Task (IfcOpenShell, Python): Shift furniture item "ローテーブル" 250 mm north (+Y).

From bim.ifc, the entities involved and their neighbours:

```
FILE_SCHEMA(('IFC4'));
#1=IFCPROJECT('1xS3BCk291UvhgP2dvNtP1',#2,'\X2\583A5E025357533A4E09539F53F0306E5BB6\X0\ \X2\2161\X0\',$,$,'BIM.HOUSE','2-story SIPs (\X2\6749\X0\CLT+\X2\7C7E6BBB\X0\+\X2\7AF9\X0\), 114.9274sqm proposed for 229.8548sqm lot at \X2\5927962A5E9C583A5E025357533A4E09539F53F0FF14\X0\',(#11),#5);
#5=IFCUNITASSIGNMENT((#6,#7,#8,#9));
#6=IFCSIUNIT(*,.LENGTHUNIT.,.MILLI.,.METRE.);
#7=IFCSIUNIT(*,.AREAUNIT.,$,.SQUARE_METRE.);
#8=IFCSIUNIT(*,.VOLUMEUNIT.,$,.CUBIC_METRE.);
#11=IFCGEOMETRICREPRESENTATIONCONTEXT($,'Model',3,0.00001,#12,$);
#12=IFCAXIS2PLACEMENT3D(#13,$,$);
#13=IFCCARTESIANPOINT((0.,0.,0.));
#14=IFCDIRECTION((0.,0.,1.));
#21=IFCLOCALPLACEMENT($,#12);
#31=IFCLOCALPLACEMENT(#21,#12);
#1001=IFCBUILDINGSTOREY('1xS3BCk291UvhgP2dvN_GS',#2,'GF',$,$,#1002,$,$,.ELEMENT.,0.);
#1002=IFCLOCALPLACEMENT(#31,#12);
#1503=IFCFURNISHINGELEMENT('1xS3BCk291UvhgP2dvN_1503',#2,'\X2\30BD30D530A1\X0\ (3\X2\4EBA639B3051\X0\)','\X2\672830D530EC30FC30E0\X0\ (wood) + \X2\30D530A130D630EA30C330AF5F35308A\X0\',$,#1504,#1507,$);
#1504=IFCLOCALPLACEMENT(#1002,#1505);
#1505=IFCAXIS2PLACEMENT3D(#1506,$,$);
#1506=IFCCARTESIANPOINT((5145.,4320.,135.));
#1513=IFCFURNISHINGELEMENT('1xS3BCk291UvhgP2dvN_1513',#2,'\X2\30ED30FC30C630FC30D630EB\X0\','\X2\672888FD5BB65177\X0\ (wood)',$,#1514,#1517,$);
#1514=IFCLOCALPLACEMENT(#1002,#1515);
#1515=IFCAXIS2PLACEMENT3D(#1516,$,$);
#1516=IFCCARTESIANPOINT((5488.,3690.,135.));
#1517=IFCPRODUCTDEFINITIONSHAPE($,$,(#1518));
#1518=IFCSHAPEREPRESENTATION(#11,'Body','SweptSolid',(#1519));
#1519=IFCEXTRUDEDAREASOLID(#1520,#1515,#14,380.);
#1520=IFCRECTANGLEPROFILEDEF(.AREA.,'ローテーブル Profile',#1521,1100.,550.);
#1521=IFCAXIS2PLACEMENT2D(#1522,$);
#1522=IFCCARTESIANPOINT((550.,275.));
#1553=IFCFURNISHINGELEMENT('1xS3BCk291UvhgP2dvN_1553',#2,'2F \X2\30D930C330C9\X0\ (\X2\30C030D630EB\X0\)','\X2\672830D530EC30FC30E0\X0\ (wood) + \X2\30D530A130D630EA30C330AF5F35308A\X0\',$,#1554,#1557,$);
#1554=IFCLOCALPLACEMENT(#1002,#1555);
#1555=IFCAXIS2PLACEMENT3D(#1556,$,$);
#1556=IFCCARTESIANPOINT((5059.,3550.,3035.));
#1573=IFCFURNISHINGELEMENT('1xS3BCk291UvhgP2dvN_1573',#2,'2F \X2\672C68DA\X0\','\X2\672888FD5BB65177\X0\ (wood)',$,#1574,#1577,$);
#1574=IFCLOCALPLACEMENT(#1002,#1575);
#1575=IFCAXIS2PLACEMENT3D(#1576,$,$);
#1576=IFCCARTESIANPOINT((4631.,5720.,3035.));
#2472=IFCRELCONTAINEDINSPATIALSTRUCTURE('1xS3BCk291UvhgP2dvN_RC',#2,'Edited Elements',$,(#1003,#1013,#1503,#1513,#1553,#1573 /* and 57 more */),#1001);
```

```python
import ifcopenshell
import ifcopenshell.api.geometry
import ifcopenshell.util.placement
import ifcopenshell.util.unit

model = ifcopenshell.open("bim.ifc")
unit_scale = ifcopenshell.util.unit.calculate_unit_scale(model)

item = model.by_id(1513)
matrix = ifcopenshell.util.placement.get_local_placement(item.ObjectPlacement)
matrix[1, 3] += 0.25 / unit_scale
ifcopenshell.api.geometry.edit_object_placement(model, product=item, matrix=matrix, is_si=False)

print(ifcopenshell.util.placement.get_local_placement(item.ObjectPlacement).round(3) + 0.0)

model.write("bim_rev.ifc")
```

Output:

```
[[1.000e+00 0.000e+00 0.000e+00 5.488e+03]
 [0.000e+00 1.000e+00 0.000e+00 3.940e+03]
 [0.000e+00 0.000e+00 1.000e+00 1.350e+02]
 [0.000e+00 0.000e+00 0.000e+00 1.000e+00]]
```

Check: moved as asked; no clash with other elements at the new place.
